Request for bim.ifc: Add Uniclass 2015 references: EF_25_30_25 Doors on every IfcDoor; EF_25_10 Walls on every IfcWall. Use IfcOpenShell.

First a look at what the model holds.

```python
import ifcopenshell

model = ifcopenshell.open("bim.ifc")
print(model.schema)
print("classifications:", [c.Name for c in model.by_type("IfcClassification")])
for ifc_class in ("IfcDoor", "IfcRoof", "IfcStair", "IfcWall", "IfcWindow"):
    print(ifc_class, len(model.by_type(ifc_class)))
```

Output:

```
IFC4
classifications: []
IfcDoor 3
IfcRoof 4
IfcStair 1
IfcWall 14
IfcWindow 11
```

```python
import ifcopenshell
import ifcopenshell.api.classification

model = ifcopenshell.open("bim.ifc")

system = ifcopenshell.api.classification.add_classification(model, classification="Uniclass 2015")

codes = {
    "IfcDoor": ("EF_25_30_25", "Doors"),
    "IfcWall": ("EF_25_10", "Walls"),
}
for ifc_class, (code, name) in codes.items():
    products = model.by_type(ifc_class)
    ifcopenshell.api.classification.add_reference(
        model, products=products, classification=system, identification=code, name=name
    )
    print(code, len(products))

model.write("bim-out.ifc")
```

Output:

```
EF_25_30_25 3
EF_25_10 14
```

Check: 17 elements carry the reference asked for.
